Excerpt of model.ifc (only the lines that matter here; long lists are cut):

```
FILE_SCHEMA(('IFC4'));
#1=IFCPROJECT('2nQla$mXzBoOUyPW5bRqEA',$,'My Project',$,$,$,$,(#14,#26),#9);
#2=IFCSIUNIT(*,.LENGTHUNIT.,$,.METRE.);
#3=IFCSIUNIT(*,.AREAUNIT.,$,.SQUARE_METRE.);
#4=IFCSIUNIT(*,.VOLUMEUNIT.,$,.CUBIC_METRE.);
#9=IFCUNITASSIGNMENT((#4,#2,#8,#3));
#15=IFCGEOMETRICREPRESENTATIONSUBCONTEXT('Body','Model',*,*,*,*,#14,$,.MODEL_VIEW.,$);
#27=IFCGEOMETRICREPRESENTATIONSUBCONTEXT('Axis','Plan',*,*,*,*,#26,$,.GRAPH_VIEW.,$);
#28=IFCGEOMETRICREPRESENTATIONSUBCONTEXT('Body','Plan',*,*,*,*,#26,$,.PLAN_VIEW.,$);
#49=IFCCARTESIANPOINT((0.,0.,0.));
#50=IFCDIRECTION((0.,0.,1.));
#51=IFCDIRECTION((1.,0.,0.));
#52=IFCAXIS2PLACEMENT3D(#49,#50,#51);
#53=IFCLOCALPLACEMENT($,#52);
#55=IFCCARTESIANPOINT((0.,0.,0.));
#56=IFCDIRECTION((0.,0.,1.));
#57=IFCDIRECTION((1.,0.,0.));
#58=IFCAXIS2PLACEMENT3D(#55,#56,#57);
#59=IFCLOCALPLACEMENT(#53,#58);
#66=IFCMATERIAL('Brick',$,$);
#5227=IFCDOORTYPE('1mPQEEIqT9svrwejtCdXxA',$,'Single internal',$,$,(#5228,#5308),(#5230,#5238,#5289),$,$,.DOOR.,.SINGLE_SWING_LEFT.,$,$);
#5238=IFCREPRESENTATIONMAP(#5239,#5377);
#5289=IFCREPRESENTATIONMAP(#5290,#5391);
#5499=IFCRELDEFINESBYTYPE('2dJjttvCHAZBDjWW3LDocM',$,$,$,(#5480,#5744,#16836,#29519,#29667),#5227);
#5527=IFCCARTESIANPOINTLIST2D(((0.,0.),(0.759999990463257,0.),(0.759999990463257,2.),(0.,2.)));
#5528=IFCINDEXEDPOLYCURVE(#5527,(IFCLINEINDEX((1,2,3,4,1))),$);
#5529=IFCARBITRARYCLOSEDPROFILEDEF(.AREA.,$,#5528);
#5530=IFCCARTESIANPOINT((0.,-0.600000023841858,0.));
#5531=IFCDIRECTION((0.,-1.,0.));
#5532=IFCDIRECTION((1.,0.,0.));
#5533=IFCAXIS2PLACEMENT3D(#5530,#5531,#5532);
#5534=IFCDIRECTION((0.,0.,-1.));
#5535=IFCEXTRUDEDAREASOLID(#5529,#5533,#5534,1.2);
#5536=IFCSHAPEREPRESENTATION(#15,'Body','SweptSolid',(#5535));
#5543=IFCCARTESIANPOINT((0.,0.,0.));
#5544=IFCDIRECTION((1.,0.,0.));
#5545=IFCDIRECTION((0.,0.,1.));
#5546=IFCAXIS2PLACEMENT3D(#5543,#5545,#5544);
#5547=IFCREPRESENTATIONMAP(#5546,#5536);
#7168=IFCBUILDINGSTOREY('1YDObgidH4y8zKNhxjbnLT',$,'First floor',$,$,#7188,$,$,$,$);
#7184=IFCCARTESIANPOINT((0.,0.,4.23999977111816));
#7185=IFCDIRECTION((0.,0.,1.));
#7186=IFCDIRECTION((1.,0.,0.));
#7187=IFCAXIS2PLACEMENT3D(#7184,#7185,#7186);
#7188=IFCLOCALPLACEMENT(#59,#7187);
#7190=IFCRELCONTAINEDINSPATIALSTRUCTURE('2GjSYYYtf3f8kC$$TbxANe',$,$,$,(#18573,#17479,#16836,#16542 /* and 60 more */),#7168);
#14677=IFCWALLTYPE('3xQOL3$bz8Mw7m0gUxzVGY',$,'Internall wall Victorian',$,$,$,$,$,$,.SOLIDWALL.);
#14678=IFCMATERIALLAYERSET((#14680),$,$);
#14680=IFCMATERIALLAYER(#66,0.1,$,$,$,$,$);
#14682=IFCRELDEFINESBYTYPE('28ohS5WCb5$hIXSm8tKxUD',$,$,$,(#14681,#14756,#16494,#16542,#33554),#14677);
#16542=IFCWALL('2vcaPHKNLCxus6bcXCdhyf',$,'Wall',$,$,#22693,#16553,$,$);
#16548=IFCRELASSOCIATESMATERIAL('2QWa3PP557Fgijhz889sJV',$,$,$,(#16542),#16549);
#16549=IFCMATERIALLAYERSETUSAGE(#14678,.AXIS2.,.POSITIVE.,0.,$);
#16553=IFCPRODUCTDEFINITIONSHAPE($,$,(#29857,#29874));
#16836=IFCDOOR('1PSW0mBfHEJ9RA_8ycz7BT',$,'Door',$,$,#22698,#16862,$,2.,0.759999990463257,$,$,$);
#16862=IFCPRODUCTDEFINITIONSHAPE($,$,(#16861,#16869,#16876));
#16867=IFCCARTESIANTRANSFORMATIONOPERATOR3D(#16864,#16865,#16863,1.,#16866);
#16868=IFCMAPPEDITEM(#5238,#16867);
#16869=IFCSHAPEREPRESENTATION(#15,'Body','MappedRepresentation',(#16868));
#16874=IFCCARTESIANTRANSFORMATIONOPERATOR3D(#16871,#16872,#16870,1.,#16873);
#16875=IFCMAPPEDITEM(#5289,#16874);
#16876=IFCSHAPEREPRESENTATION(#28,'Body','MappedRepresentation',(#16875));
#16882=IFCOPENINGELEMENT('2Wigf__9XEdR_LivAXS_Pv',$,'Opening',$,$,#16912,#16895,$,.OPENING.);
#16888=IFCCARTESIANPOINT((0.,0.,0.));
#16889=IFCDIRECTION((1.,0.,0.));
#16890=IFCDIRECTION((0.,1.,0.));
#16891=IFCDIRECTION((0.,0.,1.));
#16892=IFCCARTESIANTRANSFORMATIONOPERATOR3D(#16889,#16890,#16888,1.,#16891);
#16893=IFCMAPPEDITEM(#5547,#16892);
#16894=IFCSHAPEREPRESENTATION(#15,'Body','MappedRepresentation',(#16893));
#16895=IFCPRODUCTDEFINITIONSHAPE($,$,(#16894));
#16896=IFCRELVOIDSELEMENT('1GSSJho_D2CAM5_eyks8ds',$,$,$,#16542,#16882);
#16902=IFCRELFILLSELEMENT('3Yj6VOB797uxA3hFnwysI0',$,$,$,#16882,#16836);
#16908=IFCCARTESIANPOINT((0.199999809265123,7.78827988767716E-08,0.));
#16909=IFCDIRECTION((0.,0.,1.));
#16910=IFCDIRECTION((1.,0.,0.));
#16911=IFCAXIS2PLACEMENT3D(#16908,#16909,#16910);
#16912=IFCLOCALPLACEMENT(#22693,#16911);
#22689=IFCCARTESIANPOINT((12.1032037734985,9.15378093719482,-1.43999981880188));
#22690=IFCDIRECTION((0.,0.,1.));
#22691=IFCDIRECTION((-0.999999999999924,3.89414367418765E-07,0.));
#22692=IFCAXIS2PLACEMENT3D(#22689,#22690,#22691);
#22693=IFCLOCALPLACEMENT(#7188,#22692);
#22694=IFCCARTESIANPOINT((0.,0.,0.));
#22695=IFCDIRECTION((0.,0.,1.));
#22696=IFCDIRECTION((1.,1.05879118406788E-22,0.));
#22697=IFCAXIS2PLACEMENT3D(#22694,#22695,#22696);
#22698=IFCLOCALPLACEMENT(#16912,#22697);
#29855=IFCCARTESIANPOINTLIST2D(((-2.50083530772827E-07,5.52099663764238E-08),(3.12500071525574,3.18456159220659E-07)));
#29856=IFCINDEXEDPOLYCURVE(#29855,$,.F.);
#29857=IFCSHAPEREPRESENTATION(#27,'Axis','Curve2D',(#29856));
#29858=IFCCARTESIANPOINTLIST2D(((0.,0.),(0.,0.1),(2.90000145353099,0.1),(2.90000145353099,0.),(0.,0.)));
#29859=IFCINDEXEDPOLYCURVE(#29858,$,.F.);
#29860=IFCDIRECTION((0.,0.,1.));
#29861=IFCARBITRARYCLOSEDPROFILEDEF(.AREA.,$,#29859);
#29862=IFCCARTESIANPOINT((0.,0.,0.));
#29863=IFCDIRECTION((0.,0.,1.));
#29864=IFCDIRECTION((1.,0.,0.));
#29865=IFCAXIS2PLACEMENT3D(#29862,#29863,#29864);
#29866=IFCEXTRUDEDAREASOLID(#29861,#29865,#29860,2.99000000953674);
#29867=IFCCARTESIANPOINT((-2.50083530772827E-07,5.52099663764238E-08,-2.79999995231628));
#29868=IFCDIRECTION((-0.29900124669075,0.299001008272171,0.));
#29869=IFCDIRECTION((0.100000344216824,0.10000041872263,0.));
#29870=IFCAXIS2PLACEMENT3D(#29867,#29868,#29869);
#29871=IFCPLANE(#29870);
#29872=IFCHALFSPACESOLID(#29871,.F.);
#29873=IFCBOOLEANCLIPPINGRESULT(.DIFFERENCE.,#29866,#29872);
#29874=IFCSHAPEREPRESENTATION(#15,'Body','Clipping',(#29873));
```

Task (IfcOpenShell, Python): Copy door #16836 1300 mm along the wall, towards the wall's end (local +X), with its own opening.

```python
import ifcopenshell
import ifcopenshell.api.feature
import ifcopenshell.api.geometry
import ifcopenshell.api.root
import ifcopenshell.geom
import ifcopenshell.util.element
import ifcopenshell.util.placement
import ifcopenshell.util.shape

model = ifcopenshell.open("model.ifc")
settings = ifcopenshell.geom.settings()


def volume(element):
    """Net volume in cubic metres, openings subtracted."""
    shape = ifcopenshell.geom.create_shape(settings, element)
    return ifcopenshell.util.shape.get_volume(shape.geometry)


door = model.by_id(16836)
opening = door.FillsVoids[0].RelatingOpeningElement
wall = opening.VoidsElements[0].RelatingBuildingElement
before = volume(wall)
shift = ifcopenshell.util.placement.get_local_placement(wall.ObjectPlacement)[:3, 0] * 1.3

# copy_class copies the void relationship, type, container and properties, but no geometry.
new_opening = ifcopenshell.api.root.copy_class(model, product=opening)
new_opening.Representation = ifcopenshell.util.element.copy_deep(
    model, opening.Representation, exclude=["IfcGeometricRepresentationContext", "IfcRepresentationMap"]
)
new_door = ifcopenshell.api.root.copy_class(model, product=door)
new_door.Representation = ifcopenshell.util.element.copy_deep(
    model, door.Representation, exclude=["IfcGeometricRepresentationContext", "IfcRepresentationMap"]
)
ifcopenshell.api.feature.add_filling(model, opening=new_opening, element=new_door)

for old, new in ((opening, new_opening), (door, new_door)):
    matrix = ifcopenshell.util.placement.get_local_placement(old.ObjectPlacement)
    matrix[:3, 3] += shift
    ifcopenshell.api.geometry.edit_object_placement(model, product=new, matrix=matrix, is_si=False)

after = volume(wall)

print(f"wall volume {before:.3f} -> {after:.3f} m3")

model.write("model_edited.ifc")
```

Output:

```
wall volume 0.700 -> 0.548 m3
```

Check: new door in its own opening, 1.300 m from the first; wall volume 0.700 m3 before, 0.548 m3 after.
